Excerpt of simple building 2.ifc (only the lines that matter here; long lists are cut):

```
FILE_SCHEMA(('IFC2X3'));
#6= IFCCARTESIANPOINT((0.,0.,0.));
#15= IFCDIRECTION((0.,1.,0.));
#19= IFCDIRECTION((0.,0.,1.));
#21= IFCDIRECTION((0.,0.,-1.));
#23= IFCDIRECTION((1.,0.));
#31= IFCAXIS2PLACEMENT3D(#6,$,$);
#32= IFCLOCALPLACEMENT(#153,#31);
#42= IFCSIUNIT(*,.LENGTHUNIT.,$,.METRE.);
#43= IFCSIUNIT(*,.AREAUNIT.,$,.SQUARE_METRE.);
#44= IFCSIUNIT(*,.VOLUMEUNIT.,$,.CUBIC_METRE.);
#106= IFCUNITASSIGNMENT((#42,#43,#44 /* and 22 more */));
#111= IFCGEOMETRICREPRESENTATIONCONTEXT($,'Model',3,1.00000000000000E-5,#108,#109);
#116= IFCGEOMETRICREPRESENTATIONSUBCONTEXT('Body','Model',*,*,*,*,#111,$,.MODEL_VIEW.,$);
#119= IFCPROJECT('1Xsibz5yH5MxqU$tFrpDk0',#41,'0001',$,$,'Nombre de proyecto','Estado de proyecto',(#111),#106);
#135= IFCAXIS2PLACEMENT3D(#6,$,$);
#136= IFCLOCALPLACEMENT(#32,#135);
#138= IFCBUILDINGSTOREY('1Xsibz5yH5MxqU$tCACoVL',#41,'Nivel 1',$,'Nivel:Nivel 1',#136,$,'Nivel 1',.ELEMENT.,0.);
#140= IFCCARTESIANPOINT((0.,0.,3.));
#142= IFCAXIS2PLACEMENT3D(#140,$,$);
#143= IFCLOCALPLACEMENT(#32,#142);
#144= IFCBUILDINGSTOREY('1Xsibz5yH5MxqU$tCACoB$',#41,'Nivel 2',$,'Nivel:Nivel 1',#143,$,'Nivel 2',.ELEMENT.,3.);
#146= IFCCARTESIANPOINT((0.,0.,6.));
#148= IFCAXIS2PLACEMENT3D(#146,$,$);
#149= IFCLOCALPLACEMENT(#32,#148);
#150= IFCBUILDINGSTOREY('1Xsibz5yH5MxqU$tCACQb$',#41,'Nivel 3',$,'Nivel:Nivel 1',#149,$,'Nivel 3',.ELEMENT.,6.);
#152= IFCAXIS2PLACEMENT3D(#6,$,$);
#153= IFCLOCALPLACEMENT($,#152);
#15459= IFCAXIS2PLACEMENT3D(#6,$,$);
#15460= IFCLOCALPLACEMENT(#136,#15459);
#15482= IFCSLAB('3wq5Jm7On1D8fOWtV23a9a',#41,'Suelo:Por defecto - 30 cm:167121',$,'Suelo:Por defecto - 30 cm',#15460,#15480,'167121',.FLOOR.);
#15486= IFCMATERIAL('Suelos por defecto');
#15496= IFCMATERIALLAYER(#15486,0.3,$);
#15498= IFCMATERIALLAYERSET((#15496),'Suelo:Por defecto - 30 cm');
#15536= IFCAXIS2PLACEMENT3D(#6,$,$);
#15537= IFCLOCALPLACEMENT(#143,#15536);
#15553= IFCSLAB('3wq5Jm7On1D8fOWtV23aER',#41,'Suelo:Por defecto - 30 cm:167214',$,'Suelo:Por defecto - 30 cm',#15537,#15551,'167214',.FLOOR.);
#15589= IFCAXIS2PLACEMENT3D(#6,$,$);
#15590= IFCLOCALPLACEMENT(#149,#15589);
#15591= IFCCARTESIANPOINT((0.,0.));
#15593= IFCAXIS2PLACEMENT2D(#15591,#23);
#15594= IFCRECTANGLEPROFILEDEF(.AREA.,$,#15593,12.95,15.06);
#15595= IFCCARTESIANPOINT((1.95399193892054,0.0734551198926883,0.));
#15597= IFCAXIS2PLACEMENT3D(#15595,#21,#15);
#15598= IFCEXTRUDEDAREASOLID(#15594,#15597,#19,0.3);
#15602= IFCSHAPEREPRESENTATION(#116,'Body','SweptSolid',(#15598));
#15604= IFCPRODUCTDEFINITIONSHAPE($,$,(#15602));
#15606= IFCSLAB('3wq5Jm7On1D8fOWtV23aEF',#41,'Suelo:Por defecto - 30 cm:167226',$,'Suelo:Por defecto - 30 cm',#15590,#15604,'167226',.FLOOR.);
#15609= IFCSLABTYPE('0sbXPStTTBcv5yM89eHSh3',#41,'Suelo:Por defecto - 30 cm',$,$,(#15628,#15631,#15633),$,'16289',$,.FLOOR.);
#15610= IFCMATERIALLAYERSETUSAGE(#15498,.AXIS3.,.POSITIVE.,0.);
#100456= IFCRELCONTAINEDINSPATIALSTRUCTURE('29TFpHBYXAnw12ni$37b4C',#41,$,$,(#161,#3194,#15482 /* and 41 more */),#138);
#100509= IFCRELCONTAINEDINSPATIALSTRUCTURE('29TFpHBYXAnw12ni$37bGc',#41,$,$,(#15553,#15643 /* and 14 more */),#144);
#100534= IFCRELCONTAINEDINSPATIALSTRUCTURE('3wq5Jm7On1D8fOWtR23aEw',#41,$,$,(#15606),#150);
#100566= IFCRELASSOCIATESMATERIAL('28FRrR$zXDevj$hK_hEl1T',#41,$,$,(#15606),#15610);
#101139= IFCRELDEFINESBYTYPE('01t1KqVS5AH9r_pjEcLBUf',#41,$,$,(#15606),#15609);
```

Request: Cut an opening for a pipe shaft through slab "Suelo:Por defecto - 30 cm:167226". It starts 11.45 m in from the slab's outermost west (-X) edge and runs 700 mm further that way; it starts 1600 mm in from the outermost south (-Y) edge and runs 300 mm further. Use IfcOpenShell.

```python
import numpy as np
import ifcopenshell
import ifcopenshell.api.feature
import ifcopenshell.api.geometry
import ifcopenshell.api.root
import ifcopenshell.geom
import ifcopenshell.util.placement
import ifcopenshell.util.representation
import ifcopenshell.util.shape
import ifcopenshell.util.unit

model = ifcopenshell.open("simple building 2.ifc")
unit_scale = ifcopenshell.util.unit.calculate_unit_scale(model)
settings = ifcopenshell.geom.settings()


def volume(element):
    """Net volume in cubic metres, openings subtracted."""
    shape = ifcopenshell.geom.create_shape(settings, element)
    return ifcopenshell.util.shape.get_volume(shape.geometry)


slab = model.by_id(15606)
before = volume(slab)

# Extent in the slab's own axes, in metres. The edges named are its -X and -Y sides.
slab_shape = ifcopenshell.geom.create_shape(settings, slab)
vertices = ifcopenshell.util.shape.get_vertices(slab_shape.geometry)
x_min, y_min, bottom = vertices.min(axis=0)
top = vertices[:, 2].max()

opening = ifcopenshell.api.root.create_entity(model, ifc_class="IfcOpeningElement", name="Pipe shaft opening")
context = ifcopenshell.util.representation.get_context(model, "Model", "Body", "MODEL_VIEW")
width, depth = 0.7, 0.3
outline = [(0.0, 0.0), (width, 0.0), (width, depth), (0.0, depth), (0.0, 0.0)]
# Overshoot both faces by 50 mm so the cut is clean.
shape = ifcopenshell.api.geometry.add_slab_representation(
    model, context=context, depth=top - bottom + 0.1, polyline=outline
)
ifcopenshell.api.geometry.assign_representation(model, product=opening, representation=shape)

matrix = ifcopenshell.util.placement.get_local_placement(slab.ObjectPlacement)
matrix[:, 3] = matrix @ np.append(np.array([x_min + 11.45, y_min + 1.6, bottom - 0.05]) / unit_scale, 1.0)
ifcopenshell.api.geometry.edit_object_placement(model, product=opening, matrix=matrix, is_si=False)
ifcopenshell.api.feature.add_feature(model, feature=opening, element=slab)

after = volume(slab)

print(f"slab volume {before:.3f} -> {after:.3f} m3")

model.write("simple building 2_updated.ifc")
```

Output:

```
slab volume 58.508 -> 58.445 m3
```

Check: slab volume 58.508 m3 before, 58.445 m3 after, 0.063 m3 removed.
